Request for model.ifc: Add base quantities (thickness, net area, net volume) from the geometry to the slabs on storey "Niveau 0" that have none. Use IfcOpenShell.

First a look at what the model holds.

```python
import ifcopenshell
import ifcopenshell.util.element
import ifcopenshell.util.unit

model = ifcopenshell.open("model.ifc")
print(model.schema)
for unit_type in ("LENGTHUNIT", "AREAUNIT", "VOLUMEUNIT"):
    print(unit_type, ifcopenshell.util.unit.calculate_unit_scale(model, unit_type))
storey = next(s for s in model.by_type("IfcBuildingStorey") if s.Name == "Niveau 0")
slabs = [e for e in ifcopenshell.util.element.get_decomposition(storey) if e.is_a("IfcSlab")]
for e in sorted(slabs, key=lambda e: e.id()):
    print(e.id(), e.is_a(), e.Name, list(ifcopenshell.util.element.get_psets(e, qtos_only=True)), sep=" | ")
```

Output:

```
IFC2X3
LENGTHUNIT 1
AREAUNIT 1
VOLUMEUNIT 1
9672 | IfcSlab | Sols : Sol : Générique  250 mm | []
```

```python
import ifcopenshell
import ifcopenshell.api.pset
import ifcopenshell.geom
import ifcopenshell.util.element
import ifcopenshell.util.shape
import ifcopenshell.util.unit

model = ifcopenshell.open("model.ifc")
unit_scale = ifcopenshell.util.unit.calculate_unit_scale(model)
area_scale = ifcopenshell.util.unit.calculate_unit_scale(model, "AREAUNIT")
volume_scale = ifcopenshell.util.unit.calculate_unit_scale(model, "VOLUMEUNIT")
settings = ifcopenshell.geom.settings()

storey = next(s for s in model.by_type("IfcBuildingStorey") if s.Name == "Niveau 0")
slabs = [e for e in ifcopenshell.util.element.get_decomposition(storey) if e.is_a("IfcSlab")]

for e in sorted(slabs, key=lambda e: e.id()):
    if ifcopenshell.util.element.get_psets(e, qtos_only=True, should_inherit=False):
        continue
    # Geometry comes back in metres, in the element's own axes.
    shape = ifcopenshell.geom.create_shape(settings, e)
    values = {
        "Width": ifcopenshell.util.shape.get_z(shape.geometry) / unit_scale,
        "NetArea": ifcopenshell.util.shape.get_footprint_area(shape.geometry) / area_scale,
        "NetVolume": ifcopenshell.util.shape.get_volume(shape.geometry) / volume_scale,
    }
    qto = ifcopenshell.api.pset.add_qto(model, product=e, name="BaseQuantities")
    ifcopenshell.api.pset.edit_qto(model, qto=qto, properties=values)
    print(e.id(), {k: round(v, 3) for k, v in values.items()})

model.write("model_rev.ifc")
```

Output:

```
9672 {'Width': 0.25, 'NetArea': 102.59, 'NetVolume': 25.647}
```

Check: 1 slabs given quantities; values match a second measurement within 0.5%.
